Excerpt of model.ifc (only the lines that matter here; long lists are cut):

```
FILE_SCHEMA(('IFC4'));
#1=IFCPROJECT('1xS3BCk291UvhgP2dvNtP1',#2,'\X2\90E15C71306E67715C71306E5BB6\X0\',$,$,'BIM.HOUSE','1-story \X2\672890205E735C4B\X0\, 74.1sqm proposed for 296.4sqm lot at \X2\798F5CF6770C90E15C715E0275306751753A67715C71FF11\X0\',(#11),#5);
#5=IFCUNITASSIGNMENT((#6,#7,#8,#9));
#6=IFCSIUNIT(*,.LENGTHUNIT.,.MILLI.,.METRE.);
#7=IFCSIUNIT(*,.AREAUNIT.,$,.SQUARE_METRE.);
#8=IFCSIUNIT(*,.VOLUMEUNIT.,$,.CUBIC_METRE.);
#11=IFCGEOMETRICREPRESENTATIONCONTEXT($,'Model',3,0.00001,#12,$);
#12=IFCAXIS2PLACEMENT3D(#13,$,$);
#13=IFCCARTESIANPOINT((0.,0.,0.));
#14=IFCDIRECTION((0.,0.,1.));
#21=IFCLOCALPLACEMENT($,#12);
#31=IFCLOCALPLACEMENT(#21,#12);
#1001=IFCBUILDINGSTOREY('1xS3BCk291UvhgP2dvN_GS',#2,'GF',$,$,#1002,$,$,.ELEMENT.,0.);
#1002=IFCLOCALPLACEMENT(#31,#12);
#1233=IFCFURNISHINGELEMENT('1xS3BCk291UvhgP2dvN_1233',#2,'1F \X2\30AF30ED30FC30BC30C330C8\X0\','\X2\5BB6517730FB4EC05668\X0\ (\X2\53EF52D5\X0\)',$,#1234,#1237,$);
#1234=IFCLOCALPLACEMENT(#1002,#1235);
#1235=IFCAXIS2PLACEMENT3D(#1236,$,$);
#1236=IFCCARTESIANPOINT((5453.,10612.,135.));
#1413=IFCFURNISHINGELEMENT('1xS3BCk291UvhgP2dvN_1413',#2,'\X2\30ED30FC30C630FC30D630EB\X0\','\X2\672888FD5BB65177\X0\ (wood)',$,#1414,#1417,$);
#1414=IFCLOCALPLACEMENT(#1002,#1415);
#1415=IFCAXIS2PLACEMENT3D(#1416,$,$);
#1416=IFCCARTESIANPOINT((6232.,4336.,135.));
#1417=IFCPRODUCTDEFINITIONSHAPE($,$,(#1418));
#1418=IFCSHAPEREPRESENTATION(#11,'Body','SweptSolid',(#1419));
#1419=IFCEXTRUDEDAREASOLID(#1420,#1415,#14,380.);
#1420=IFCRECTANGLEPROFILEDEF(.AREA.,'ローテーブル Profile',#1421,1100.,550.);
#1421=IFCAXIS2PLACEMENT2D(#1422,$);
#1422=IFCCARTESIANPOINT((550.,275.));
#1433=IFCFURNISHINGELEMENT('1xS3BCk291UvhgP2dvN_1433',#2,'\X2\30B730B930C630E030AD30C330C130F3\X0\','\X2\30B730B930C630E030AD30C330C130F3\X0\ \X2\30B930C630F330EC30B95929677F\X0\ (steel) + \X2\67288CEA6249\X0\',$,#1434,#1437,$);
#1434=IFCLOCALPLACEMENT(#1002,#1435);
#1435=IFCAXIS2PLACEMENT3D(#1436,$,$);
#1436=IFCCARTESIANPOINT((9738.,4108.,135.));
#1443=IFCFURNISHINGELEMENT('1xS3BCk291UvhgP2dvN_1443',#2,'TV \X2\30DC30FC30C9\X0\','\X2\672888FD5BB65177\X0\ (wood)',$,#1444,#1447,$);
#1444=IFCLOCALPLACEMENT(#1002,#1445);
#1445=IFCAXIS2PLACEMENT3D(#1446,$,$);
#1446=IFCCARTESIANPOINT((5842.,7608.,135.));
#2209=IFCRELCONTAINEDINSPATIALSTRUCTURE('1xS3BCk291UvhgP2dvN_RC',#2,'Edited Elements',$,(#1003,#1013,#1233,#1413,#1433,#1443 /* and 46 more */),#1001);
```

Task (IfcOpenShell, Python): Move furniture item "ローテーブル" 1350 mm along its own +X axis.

```python
import ifcopenshell
import ifcopenshell.api.geometry
import ifcopenshell.util.placement
import ifcopenshell.util.unit

model = ifcopenshell.open("model.ifc")
unit_scale = ifcopenshell.util.unit.calculate_unit_scale(model)

item = model.by_guid("1xS3BCk291UvhgP2dvN_1413")
matrix = ifcopenshell.util.placement.get_local_placement(item.ObjectPlacement)
matrix[:3, 3] += matrix[:3, 0] * 1.35 / unit_scale
ifcopenshell.api.geometry.edit_object_placement(model, product=item, matrix=matrix, is_si=False)

print(ifcopenshell.util.placement.get_local_placement(item.ObjectPlacement).round(3) + 0.0)

model.write("model-out.ifc")
```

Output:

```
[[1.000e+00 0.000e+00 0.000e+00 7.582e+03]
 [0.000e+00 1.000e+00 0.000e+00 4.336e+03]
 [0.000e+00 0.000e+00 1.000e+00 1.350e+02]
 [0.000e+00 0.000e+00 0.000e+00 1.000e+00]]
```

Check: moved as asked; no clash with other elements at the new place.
